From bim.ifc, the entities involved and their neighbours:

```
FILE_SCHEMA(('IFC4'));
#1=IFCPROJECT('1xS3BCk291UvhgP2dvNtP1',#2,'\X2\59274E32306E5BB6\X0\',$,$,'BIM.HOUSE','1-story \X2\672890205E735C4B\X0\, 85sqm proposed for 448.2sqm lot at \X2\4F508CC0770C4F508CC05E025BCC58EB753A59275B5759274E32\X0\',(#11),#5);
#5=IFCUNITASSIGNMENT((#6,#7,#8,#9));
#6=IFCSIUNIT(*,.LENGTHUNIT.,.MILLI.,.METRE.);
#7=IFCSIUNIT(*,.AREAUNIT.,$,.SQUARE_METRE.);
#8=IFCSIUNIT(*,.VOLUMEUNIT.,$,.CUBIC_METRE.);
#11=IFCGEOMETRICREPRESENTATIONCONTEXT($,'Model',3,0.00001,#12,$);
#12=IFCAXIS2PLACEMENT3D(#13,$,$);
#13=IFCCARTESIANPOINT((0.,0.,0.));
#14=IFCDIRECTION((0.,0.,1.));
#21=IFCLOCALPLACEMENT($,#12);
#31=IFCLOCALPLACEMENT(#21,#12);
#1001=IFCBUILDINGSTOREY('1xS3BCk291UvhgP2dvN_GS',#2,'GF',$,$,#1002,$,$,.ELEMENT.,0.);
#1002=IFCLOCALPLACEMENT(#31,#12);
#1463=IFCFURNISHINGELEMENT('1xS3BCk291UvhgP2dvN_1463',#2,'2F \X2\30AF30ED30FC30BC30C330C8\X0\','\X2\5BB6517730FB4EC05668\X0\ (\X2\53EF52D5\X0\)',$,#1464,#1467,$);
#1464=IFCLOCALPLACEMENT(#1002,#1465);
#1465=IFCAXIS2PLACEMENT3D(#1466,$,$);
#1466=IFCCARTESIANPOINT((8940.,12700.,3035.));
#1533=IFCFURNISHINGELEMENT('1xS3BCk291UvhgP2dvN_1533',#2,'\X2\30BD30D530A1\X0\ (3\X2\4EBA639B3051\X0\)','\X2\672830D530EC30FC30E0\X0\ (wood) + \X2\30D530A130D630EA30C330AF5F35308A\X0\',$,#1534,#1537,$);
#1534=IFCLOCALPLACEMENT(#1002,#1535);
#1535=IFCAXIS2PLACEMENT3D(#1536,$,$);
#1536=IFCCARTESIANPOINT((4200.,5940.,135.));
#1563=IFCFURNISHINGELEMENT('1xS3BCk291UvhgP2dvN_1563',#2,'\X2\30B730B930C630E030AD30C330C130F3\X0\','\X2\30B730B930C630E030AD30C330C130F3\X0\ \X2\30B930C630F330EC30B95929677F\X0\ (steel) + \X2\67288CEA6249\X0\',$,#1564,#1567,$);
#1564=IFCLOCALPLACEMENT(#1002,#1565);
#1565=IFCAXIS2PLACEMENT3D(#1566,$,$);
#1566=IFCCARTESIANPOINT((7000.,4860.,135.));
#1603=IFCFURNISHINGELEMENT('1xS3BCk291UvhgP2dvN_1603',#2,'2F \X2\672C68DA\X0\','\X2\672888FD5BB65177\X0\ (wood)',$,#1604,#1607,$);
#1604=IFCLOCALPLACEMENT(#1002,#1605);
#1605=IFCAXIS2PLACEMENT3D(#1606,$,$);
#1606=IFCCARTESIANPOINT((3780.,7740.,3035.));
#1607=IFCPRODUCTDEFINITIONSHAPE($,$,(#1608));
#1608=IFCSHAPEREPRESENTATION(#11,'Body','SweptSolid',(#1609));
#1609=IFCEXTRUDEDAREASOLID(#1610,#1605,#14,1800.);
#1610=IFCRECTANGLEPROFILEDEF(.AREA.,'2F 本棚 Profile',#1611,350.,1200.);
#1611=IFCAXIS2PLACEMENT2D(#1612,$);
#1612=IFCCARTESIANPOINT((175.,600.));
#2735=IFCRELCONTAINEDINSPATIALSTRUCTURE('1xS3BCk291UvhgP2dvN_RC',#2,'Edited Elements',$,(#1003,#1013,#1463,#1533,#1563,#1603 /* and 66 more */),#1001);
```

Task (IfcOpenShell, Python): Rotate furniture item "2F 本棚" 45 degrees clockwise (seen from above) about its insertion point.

```python
import ifcopenshell
import ifcopenshell.api.geometry
import ifcopenshell.util.placement

model = ifcopenshell.open("bim.ifc")

item = model.by_guid("1xS3BCk291UvhgP2dvN_1603")
matrix = ifcopenshell.util.placement.get_local_placement(item.ObjectPlacement)
matrix = matrix @ ifcopenshell.util.placement.rotation(-45, "Z")
ifcopenshell.api.geometry.edit_object_placement(model, product=item, matrix=matrix, is_si=False)

print(ifcopenshell.util.placement.get_local_placement(item.ObjectPlacement).round(3) + 0.0)

model.write("bim-out.ifc")
```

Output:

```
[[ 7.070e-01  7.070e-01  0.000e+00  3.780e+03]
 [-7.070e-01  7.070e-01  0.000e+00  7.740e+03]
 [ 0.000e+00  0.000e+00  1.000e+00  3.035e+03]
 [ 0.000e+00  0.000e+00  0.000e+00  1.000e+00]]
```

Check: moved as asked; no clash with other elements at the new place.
